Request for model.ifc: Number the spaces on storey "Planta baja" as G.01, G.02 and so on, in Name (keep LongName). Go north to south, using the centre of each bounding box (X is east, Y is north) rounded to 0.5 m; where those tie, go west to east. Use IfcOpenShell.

First a look at what the model holds.

```python
import ifcopenshell
import ifcopenshell.util.element
import ifcopenshell.util.placement

model = ifcopenshell.open("model.ifc")
print(model.schema)
storey = next(s for s in model.by_type("IfcBuildingStorey") if s.Name == "Planta baja")
spaces = [e for e in ifcopenshell.util.element.get_decomposition(storey) if e.is_a("IfcSpace")]
for e in sorted(spaces, key=lambda e: e.id()):
    origin = ifcopenshell.util.placement.get_local_placement(e.ObjectPlacement)[:3, 3]
    print(e.id(), e.Name, e.LongName, origin.round(2) + 0.0, sep=" | ")
```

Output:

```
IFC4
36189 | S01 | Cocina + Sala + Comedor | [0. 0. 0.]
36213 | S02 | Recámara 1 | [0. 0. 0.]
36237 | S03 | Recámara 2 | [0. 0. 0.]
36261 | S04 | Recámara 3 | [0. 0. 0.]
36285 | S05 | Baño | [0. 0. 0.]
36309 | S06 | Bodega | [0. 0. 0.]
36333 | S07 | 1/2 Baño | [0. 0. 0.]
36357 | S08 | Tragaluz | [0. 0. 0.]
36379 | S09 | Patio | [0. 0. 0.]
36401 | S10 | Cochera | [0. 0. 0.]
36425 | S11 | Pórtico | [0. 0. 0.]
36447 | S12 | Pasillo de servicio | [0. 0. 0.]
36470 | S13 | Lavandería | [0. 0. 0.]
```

```python
import ifcopenshell
import ifcopenshell.geom
import ifcopenshell.util.element
import ifcopenshell.util.shape

model = ifcopenshell.open("model.ifc")
settings = ifcopenshell.geom.settings()
settings.set("use-world-coords", True)


def centre(element):
    shape = ifcopenshell.geom.create_shape(settings, element)
    return ifcopenshell.util.shape.get_bbox_centroid(shape.geometry)


storey = next(s for s in model.by_type("IfcBuildingStorey") if s.Name == "Planta baja")
spaces = [e for e in ifcopenshell.util.element.get_decomposition(storey) if e.is_a("IfcSpace")]

# Insertion points can sit at a corner or the storey origin, so sort by the geometry (in metres).
centres = {e: centre(e) for e in spaces}
spaces.sort(key=lambda e: (-round(centres[e][1] / 0.5), centres[e][0]))

for i, e in enumerate(spaces, start=1):
    number = f"G.{i:02d}"
    e.Name = number
    print(e.id(), number)

model.write("model_updated.ifc")
```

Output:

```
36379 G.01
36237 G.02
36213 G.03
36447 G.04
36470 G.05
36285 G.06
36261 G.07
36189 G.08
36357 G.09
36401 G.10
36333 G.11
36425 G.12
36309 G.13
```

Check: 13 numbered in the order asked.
